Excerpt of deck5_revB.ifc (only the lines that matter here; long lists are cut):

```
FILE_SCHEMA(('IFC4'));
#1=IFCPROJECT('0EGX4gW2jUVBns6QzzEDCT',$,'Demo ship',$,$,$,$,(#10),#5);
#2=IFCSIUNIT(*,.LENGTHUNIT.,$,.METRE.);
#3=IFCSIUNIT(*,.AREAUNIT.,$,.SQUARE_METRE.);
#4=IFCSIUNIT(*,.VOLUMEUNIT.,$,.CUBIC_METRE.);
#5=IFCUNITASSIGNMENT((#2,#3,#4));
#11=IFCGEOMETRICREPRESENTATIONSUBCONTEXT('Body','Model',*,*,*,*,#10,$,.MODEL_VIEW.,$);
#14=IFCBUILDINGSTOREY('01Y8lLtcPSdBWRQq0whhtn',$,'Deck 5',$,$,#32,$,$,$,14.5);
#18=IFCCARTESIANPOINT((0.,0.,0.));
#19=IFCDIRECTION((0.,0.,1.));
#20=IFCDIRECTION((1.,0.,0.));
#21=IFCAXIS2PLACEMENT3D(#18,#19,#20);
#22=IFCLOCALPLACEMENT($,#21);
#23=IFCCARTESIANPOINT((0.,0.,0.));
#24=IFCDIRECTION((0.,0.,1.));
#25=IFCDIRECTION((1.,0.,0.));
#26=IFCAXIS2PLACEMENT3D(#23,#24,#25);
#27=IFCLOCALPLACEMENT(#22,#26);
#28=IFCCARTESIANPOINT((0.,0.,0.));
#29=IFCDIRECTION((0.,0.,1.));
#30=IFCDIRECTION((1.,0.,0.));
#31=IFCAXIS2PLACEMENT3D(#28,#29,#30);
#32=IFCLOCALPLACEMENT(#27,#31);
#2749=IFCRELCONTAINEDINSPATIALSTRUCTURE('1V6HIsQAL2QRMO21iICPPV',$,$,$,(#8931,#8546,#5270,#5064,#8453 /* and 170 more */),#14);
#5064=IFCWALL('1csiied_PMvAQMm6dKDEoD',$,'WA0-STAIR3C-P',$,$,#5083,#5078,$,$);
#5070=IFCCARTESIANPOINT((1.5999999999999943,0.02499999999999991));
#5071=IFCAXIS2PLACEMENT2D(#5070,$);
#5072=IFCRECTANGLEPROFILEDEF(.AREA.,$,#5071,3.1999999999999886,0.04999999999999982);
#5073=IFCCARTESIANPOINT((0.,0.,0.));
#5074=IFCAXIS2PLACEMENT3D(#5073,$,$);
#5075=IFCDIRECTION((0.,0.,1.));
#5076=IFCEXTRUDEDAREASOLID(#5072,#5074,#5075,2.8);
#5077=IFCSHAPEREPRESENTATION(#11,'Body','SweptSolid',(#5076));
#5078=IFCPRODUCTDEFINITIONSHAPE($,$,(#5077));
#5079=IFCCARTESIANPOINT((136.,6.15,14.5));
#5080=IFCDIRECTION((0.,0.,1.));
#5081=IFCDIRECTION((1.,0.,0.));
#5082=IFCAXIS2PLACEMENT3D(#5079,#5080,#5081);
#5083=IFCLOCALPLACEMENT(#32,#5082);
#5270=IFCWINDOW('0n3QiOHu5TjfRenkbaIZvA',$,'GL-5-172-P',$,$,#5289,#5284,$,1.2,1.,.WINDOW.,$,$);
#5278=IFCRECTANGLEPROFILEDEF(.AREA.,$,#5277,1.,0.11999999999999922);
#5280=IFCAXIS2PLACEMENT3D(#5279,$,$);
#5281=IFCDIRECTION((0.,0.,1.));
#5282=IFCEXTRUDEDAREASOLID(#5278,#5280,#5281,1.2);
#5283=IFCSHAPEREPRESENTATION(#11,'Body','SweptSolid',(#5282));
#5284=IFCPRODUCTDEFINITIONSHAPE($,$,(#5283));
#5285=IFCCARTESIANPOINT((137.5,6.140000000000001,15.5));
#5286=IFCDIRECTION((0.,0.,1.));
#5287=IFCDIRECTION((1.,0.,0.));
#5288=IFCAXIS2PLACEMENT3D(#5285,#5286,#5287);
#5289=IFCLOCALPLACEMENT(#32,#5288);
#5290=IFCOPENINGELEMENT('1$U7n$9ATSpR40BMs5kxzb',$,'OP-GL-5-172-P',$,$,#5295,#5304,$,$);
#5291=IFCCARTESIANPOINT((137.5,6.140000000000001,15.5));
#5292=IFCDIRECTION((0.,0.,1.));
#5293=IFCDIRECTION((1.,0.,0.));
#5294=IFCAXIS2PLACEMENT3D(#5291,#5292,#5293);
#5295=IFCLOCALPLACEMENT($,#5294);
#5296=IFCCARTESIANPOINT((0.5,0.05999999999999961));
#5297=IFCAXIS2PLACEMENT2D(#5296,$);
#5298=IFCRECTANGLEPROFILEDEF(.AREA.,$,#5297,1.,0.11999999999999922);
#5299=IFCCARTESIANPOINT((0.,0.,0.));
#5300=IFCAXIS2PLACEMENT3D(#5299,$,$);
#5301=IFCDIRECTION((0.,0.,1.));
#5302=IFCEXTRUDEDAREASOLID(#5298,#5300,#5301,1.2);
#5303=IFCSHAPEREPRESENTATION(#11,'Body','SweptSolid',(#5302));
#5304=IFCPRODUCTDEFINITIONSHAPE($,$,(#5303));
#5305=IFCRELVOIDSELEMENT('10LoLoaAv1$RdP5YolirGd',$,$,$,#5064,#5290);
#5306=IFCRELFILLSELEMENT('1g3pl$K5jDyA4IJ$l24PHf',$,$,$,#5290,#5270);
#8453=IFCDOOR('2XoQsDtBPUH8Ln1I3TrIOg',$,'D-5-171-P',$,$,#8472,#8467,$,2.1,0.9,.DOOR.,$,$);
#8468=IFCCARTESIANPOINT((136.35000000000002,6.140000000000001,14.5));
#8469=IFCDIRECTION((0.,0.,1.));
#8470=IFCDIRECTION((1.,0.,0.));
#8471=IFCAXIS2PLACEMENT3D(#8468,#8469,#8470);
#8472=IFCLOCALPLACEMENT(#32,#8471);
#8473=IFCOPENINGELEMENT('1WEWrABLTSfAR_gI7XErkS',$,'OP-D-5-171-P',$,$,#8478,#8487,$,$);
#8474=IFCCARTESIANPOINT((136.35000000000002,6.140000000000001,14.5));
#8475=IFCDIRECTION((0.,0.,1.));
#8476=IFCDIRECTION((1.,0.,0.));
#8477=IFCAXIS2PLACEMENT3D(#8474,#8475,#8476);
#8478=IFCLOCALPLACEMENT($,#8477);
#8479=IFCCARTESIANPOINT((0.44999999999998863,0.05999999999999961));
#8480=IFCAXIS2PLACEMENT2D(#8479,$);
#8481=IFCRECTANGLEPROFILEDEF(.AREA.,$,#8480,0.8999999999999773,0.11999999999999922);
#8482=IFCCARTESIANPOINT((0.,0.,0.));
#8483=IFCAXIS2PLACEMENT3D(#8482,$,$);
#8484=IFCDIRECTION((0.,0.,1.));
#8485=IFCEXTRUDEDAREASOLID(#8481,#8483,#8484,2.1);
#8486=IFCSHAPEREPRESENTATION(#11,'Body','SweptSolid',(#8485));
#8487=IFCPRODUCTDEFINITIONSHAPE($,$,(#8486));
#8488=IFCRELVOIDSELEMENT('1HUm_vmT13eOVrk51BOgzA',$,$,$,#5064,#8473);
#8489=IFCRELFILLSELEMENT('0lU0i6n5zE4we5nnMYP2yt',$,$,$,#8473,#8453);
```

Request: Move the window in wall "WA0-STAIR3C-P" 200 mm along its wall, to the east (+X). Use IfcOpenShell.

```python
import ifcopenshell
import ifcopenshell.api.geometry
import ifcopenshell.util.placement
import ifcopenshell.util.unit

model = ifcopenshell.open("deck5_revB.ifc")
unit_scale = ifcopenshell.util.unit.calculate_unit_scale(model)

window = model.by_guid("0n3QiOHu5TjfRenkbaIZvA")
opening = window.FillsVoids[0].RelatingOpeningElement
wall = opening.VoidsElements[0].RelatingBuildingElement

wall_matrix = ifcopenshell.util.placement.get_local_placement(wall.ObjectPlacement)
shift = wall_matrix[:3, 0] * 0.2 / unit_scale
before = ifcopenshell.util.placement.get_local_placement(window.ObjectPlacement)[:3, 3].copy()

# The window is not placed relative to its opening, so move both.
for product in (opening, window):
    matrix = ifcopenshell.util.placement.get_local_placement(product.ObjectPlacement)
    matrix[:3, 3] += shift
    ifcopenshell.api.geometry.edit_object_placement(model, product=product, matrix=matrix, is_si=False)

after = ifcopenshell.util.placement.get_local_placement(window.ObjectPlacement)[:3, 3]
print("window moved by", (after - before).round(3) + 0.0)

model.write("deck5_revB_v2.ifc")
```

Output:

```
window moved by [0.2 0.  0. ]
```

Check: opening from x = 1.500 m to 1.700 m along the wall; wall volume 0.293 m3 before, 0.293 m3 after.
